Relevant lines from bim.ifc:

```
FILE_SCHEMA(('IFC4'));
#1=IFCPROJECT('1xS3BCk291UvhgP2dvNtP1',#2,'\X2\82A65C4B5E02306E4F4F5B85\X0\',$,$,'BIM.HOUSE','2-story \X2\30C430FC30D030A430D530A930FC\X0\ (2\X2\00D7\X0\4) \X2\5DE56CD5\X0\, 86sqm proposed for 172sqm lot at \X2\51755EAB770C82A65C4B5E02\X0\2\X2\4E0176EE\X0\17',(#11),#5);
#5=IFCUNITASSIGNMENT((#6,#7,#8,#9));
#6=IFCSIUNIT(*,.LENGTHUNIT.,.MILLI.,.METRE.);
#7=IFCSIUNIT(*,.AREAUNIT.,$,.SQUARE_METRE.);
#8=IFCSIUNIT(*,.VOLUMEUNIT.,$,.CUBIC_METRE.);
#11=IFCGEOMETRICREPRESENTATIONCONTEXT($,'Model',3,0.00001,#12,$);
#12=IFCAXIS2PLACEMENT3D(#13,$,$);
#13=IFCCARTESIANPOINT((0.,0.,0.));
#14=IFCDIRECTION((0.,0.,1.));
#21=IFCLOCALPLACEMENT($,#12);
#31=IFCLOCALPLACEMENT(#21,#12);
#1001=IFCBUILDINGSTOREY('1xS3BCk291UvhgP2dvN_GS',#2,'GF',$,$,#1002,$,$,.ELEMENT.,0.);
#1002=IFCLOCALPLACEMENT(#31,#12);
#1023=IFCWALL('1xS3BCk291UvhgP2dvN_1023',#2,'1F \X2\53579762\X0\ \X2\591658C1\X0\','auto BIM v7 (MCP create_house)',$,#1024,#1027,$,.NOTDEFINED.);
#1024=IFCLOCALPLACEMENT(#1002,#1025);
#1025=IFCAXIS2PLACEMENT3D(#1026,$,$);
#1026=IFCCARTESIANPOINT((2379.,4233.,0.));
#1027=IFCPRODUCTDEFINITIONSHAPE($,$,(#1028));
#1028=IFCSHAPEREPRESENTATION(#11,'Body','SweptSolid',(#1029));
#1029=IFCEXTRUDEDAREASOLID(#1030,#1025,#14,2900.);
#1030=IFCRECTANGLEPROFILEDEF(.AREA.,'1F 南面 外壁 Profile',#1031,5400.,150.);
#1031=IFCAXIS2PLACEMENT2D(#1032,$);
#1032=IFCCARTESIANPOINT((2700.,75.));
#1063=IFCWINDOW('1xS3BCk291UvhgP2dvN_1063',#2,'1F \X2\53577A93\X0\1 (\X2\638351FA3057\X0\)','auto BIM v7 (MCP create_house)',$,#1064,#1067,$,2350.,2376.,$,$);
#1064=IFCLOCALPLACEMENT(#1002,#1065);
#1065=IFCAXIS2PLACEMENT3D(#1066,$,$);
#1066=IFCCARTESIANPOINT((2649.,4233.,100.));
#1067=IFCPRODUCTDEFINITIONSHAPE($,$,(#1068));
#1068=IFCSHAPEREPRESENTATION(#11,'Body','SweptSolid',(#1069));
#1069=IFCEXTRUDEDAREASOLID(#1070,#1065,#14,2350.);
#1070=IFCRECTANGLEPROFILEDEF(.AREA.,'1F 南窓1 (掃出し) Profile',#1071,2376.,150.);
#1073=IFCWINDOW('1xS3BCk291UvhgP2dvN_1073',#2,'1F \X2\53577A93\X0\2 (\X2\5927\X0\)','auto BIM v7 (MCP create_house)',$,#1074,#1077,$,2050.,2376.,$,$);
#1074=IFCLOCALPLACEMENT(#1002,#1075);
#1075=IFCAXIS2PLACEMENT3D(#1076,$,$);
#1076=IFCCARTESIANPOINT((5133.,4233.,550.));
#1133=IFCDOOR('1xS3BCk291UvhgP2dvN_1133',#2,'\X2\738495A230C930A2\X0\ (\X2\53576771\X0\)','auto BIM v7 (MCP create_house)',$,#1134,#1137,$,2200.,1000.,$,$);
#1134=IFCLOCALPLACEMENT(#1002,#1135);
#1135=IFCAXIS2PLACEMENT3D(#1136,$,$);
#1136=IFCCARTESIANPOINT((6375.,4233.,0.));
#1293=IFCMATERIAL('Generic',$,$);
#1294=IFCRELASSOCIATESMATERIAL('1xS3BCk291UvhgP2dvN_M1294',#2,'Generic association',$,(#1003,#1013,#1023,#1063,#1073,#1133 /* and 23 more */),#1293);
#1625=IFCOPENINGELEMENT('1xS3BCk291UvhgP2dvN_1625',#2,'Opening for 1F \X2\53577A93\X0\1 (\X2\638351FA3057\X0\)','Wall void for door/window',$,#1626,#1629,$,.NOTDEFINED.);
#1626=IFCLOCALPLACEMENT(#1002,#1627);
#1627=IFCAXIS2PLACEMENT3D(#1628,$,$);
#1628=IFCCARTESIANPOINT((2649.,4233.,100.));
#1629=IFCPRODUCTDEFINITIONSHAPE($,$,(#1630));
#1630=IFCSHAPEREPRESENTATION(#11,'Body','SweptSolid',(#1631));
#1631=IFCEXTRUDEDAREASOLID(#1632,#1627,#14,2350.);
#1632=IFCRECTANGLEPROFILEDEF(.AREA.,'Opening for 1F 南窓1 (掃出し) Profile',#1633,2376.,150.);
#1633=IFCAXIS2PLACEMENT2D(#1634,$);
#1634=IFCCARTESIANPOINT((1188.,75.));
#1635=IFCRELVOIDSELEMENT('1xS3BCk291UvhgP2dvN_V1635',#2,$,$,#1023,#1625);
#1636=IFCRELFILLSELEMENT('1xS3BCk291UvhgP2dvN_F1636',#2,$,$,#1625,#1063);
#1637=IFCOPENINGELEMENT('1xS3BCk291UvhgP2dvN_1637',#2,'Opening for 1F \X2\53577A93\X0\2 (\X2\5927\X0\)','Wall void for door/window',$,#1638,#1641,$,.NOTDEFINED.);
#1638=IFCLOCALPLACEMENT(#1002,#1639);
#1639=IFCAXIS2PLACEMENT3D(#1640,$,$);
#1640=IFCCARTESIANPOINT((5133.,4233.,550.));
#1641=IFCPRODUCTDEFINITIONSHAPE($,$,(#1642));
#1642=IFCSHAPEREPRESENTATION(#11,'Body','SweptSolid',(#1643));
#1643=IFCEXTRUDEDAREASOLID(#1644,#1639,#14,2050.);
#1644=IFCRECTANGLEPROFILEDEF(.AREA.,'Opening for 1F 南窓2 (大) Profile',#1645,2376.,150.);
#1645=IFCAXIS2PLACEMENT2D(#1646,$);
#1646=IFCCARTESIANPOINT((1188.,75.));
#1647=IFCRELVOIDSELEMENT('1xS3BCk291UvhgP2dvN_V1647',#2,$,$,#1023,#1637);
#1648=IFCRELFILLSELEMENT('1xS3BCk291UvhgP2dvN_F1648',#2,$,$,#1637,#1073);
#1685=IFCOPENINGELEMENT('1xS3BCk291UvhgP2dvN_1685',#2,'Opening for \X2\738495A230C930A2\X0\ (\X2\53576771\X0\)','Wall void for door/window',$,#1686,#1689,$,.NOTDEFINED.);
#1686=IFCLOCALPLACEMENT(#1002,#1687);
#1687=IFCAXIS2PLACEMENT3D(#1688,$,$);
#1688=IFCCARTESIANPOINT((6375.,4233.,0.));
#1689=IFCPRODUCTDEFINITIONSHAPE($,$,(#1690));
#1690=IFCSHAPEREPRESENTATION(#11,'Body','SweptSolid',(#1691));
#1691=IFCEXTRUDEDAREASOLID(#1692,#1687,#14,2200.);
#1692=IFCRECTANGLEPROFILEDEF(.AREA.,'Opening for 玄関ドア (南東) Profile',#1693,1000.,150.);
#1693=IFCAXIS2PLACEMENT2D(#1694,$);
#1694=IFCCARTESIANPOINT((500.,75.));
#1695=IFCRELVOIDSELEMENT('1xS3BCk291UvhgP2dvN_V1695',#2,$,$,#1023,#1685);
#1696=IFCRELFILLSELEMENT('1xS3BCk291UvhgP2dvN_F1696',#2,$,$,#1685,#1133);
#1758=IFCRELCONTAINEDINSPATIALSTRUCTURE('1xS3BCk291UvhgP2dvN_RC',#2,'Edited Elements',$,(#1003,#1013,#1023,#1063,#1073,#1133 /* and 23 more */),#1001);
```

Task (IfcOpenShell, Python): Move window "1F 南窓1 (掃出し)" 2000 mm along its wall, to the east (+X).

```python
import ifcopenshell
import ifcopenshell.api.geometry
import ifcopenshell.util.placement
import ifcopenshell.util.unit

model = ifcopenshell.open("bim.ifc")
unit_scale = ifcopenshell.util.unit.calculate_unit_scale(model)

window = model.by_guid("1xS3BCk291UvhgP2dvN_1063")
opening = window.FillsVoids[0].RelatingOpeningElement
wall = opening.VoidsElements[0].RelatingBuildingElement

wall_matrix = ifcopenshell.util.placement.get_local_placement(wall.ObjectPlacement)
shift = wall_matrix[:3, 0] * 2 / unit_scale
before = ifcopenshell.util.placement.get_local_placement(window.ObjectPlacement)[:3, 3].copy()

# The window is not placed relative to its opening, so move both.
for product in (opening, window):
    matrix = ifcopenshell.util.placement.get_local_placement(product.ObjectPlacement)
    matrix[:3, 3] += shift
    ifcopenshell.api.geometry.edit_object_placement(model, product=product, matrix=matrix, is_si=False)

after = ifcopenshell.util.placement.get_local_placement(window.ObjectPlacement)[:3, 3]
print("window moved by", (after - before).round(3) + 0.0)

model.write("bim-out.ifc")
```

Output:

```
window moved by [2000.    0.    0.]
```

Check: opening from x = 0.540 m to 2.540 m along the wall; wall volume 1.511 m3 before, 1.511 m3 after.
